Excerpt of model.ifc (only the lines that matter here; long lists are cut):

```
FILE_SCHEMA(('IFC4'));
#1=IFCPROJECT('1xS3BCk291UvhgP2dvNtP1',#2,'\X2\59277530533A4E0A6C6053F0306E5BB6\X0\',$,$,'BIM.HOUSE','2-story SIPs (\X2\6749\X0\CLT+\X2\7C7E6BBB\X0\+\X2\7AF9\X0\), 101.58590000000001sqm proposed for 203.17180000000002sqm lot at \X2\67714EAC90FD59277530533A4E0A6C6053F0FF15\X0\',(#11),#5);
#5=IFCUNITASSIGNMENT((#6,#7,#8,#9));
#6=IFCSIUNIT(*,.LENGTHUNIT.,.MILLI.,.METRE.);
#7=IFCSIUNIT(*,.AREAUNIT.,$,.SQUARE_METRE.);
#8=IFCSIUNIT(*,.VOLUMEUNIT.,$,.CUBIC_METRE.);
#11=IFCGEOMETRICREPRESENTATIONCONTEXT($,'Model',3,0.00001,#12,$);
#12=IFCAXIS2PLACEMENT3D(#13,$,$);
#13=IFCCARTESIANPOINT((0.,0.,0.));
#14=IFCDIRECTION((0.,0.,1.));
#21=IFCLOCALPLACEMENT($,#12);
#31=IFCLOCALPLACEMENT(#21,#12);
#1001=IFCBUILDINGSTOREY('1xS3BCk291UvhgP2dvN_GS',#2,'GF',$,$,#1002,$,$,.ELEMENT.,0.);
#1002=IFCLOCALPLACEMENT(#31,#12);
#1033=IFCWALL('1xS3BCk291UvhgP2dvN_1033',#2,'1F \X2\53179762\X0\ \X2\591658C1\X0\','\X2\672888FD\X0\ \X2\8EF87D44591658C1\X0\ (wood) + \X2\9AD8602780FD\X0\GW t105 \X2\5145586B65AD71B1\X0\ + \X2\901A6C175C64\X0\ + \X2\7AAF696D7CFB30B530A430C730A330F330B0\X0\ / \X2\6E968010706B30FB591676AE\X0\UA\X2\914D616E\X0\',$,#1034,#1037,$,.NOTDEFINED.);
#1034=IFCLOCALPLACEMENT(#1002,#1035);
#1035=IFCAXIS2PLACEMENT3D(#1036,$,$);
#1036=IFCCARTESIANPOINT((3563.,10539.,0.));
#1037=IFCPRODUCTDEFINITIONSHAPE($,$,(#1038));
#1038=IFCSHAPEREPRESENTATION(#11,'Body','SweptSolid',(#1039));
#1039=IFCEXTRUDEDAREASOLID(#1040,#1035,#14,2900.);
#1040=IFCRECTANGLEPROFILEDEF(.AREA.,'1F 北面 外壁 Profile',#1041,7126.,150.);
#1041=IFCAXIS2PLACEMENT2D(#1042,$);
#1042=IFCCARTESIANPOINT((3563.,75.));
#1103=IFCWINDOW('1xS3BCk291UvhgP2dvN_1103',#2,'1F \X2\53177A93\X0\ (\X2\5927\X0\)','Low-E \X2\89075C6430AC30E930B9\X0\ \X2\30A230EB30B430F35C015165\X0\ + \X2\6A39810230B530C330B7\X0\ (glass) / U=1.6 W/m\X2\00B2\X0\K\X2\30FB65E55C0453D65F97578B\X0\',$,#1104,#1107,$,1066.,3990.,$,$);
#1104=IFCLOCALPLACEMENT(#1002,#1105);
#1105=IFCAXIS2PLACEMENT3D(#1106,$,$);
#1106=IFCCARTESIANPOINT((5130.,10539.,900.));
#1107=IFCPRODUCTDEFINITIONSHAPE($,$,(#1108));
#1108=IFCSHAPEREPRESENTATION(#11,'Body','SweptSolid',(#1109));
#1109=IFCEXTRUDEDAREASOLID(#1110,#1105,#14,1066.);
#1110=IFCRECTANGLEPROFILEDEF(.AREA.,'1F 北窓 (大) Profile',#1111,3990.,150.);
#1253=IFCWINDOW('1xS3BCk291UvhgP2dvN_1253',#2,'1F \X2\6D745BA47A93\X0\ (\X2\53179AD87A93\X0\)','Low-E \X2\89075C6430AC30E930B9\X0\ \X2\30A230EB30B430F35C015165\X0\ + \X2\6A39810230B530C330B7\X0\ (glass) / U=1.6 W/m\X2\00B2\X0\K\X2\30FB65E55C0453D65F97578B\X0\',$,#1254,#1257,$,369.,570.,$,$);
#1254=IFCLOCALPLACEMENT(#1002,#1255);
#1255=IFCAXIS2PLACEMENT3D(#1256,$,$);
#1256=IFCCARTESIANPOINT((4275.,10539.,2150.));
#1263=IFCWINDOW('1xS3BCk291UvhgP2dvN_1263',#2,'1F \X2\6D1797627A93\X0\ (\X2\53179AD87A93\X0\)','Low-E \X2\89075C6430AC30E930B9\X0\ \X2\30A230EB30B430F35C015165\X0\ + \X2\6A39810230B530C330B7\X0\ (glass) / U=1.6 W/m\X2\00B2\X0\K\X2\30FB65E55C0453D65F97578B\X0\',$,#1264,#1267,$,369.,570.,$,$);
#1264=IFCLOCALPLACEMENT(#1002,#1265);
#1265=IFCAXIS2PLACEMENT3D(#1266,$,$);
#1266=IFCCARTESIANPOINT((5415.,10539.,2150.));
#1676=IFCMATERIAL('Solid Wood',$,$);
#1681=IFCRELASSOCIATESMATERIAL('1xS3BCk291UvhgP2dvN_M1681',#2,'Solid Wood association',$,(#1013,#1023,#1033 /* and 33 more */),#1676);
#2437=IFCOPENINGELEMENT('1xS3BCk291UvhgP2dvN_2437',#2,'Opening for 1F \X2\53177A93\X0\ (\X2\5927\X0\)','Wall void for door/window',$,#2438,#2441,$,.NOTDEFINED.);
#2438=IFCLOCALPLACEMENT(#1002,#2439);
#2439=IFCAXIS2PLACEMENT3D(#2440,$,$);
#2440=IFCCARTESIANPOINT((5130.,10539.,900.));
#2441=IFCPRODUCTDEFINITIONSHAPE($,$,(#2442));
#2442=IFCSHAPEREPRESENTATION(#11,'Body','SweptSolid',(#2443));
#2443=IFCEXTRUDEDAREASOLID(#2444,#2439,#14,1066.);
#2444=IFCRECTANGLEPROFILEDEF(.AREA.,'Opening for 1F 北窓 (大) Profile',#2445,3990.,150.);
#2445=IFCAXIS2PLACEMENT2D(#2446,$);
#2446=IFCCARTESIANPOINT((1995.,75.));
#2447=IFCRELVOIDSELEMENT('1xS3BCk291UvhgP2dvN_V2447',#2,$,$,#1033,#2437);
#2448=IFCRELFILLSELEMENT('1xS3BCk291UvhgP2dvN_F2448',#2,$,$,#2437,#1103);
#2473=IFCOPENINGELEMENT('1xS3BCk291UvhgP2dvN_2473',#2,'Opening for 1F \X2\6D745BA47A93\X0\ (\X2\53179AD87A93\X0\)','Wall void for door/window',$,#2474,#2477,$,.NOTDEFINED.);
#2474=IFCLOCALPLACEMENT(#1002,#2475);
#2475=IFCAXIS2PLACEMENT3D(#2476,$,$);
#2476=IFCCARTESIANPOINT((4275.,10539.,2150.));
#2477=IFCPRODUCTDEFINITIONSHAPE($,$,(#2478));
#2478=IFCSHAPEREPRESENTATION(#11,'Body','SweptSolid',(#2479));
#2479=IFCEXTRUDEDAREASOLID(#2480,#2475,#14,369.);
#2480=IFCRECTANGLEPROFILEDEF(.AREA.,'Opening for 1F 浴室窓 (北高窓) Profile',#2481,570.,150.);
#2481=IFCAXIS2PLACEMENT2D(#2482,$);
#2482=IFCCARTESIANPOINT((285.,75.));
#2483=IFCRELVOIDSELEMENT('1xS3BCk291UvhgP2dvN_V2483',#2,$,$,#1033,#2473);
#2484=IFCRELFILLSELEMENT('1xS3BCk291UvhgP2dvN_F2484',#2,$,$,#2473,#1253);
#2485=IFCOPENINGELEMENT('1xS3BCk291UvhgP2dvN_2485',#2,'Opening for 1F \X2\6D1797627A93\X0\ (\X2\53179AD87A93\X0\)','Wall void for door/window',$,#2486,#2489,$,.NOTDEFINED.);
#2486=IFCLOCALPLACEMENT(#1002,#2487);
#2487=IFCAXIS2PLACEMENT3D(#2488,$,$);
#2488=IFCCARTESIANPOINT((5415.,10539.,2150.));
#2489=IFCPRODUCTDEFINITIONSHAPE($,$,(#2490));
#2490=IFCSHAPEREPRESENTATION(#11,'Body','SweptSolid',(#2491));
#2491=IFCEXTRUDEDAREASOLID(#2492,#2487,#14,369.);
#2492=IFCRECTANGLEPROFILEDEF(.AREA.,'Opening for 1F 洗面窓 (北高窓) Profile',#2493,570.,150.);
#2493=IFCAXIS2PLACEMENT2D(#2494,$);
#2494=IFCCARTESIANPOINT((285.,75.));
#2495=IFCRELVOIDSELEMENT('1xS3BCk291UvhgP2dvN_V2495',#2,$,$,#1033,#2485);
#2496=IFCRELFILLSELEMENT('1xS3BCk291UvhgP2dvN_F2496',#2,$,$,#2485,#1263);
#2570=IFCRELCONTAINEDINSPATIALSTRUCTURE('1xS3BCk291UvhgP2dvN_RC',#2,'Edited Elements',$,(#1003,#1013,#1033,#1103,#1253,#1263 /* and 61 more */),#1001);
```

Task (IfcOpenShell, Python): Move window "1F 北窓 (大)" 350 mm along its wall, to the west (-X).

```python
import ifcopenshell
import ifcopenshell.api.geometry
import ifcopenshell.util.placement
import ifcopenshell.util.unit

model = ifcopenshell.open("model.ifc")
unit_scale = ifcopenshell.util.unit.calculate_unit_scale(model)

window = model.by_guid("1xS3BCk291UvhgP2dvN_1103")
opening = window.FillsVoids[0].RelatingOpeningElement
wall = opening.VoidsElements[0].RelatingBuildingElement

wall_matrix = ifcopenshell.util.placement.get_local_placement(wall.ObjectPlacement)
shift = wall_matrix[:3, 0] * -0.35 / unit_scale
before = ifcopenshell.util.placement.get_local_placement(window.ObjectPlacement)[:3, 3].copy()

# The window is not placed relative to its opening, so move both.
for product in (opening, window):
    matrix = ifcopenshell.util.placement.get_local_placement(product.ObjectPlacement)
    matrix[:3, 3] += shift
    ifcopenshell.api.geometry.edit_object_placement(model, product=product, matrix=matrix, is_si=False)

after = ifcopenshell.util.placement.get_local_placement(window.ObjectPlacement)[:3, 3]
print("window moved by", (after - before).round(3) + 0.0)

model.write("model-out.ifc")
```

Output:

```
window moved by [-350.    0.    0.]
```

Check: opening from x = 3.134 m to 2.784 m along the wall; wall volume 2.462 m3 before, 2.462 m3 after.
